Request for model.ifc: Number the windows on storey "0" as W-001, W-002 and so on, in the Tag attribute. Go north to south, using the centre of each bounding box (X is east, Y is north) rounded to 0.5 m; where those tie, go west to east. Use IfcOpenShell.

First a look at what the model holds.

```python
import ifcopenshell
import ifcopenshell.util.element
import ifcopenshell.util.placement

model = ifcopenshell.open("model.ifc")
print(model.schema)
storey = next(s for s in model.by_type("IfcBuildingStorey") if s.Name == "0")
windows = [e for e in ifcopenshell.util.element.get_decomposition(storey) if e.is_a("IfcWindow")]
for e in sorted(windows, key=lambda e: e.id()):
    origin = ifcopenshell.util.placement.get_local_placement(e.ObjectPlacement)[:3, 3]
    print(e.id(), e.Tag, e.Name, origin.round(2) + 0.0, sep=" | ")
```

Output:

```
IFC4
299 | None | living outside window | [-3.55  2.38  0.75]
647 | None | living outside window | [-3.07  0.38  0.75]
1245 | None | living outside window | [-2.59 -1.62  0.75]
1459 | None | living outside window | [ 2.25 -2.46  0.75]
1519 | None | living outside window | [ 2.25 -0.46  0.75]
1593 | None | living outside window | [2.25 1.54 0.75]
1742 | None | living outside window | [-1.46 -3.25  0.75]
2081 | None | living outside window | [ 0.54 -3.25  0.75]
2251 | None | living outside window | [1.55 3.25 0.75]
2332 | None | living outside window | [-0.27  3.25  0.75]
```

```python
import ifcopenshell
import ifcopenshell.geom
import ifcopenshell.util.element
import ifcopenshell.util.shape

model = ifcopenshell.open("model.ifc")
settings = ifcopenshell.geom.settings()
settings.set("use-world-coords", True)


def centre(element):
    shape = ifcopenshell.geom.create_shape(settings, element)
    return ifcopenshell.util.shape.get_bbox_centroid(shape.geometry)


storey = next(s for s in model.by_type("IfcBuildingStorey") if s.Name == "0")
windows = [e for e in ifcopenshell.util.element.get_decomposition(storey) if e.is_a("IfcWindow")]

# Insertion points can sit at a corner or the storey origin, so sort by the geometry (in metres).
centres = {e: centre(e) for e in windows}
windows.sort(key=lambda e: (-round(centres[e][1] / 0.5), centres[e][0]))

for i, e in enumerate(windows, start=1):
    number = f"W-0{i:02d}"
    e.Tag = number
    print(e.id(), number)

model.write("model_updated.ifc")
```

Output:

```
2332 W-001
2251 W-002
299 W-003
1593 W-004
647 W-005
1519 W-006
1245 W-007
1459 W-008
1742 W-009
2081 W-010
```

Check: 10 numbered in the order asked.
